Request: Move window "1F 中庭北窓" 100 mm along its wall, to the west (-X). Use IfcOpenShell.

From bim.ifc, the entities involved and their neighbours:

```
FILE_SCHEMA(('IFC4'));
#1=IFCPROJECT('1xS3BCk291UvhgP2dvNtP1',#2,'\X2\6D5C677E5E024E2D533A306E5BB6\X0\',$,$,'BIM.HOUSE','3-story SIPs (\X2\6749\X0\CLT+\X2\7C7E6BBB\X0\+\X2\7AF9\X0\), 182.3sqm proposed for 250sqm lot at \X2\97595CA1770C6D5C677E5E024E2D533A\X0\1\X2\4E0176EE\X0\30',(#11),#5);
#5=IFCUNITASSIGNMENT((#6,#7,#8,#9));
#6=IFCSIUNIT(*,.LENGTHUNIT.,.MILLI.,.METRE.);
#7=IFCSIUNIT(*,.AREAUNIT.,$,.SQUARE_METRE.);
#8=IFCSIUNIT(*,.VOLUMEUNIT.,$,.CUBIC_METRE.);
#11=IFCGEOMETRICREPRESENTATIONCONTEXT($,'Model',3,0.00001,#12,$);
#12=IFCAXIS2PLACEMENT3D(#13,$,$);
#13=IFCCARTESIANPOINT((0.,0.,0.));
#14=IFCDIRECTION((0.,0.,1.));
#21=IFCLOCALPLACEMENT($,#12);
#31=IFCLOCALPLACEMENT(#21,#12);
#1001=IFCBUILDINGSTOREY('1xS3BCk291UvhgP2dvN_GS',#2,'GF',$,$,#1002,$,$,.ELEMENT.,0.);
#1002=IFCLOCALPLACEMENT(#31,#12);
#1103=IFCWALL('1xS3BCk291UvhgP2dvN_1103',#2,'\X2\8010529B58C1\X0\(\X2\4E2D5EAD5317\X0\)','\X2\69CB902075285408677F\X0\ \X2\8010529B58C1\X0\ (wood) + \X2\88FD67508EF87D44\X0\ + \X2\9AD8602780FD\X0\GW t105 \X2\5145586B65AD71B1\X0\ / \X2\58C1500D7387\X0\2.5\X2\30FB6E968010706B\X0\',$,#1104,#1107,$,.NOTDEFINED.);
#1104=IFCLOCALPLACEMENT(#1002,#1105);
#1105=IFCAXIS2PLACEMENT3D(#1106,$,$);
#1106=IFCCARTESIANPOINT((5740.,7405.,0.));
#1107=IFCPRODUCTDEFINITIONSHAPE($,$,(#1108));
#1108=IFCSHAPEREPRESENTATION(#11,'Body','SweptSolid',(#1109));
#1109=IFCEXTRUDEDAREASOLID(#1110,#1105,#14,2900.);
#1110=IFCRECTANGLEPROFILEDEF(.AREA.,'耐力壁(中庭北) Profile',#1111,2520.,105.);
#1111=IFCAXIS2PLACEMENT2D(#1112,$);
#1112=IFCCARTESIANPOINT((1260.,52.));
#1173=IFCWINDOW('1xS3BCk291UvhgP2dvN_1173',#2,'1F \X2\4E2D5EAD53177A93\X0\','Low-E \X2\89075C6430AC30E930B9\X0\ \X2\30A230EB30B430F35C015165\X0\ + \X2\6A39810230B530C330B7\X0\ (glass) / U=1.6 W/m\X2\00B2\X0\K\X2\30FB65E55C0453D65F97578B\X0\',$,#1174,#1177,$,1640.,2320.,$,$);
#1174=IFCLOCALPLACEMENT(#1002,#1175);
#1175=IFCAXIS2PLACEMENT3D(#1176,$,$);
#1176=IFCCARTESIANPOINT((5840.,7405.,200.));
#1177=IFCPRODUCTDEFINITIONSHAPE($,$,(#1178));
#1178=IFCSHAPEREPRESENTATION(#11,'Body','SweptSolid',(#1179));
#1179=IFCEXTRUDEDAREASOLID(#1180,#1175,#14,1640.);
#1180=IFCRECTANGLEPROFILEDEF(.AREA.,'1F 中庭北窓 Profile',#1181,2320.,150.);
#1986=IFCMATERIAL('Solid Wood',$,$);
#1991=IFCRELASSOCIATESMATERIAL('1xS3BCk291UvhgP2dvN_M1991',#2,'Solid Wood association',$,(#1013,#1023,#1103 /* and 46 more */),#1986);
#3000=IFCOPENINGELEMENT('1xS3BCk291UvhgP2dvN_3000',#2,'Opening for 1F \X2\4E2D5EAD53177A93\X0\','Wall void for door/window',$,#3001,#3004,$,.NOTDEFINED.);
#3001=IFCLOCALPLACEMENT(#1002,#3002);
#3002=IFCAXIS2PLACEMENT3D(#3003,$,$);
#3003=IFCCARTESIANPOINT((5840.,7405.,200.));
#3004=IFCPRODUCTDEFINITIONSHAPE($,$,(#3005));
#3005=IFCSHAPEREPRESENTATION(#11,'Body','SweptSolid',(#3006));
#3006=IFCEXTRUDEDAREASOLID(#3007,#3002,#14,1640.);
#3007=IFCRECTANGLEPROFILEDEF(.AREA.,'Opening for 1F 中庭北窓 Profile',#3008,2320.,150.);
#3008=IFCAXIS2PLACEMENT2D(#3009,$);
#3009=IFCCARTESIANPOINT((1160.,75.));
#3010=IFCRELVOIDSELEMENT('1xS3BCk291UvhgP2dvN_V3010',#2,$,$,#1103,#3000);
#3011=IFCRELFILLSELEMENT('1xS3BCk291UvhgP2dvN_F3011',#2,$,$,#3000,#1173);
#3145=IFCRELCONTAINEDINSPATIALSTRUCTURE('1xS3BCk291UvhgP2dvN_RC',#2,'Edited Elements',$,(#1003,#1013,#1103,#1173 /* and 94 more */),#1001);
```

```python
import ifcopenshell
import ifcopenshell.api.geometry
import ifcopenshell.util.placement

model = ifcopenshell.open("bim.ifc")

window = model.by_id(1173)
opening = window.FillsVoids[0].RelatingOpeningElement
wall = opening.VoidsElements[0].RelatingBuildingElement

wall_matrix = ifcopenshell.util.placement.get_local_placement(wall.ObjectPlacement)
shift = wall_matrix[:3, 0] * -100.0
before = ifcopenshell.util.placement.get_local_placement(window.ObjectPlacement)[:3, 3].copy()

# The window is not placed relative to its opening, so move both.
for product in (opening, window):
    matrix = ifcopenshell.util.placement.get_local_placement(product.ObjectPlacement)
    matrix[:3, 3] += shift
    ifcopenshell.api.geometry.edit_object_placement(model, product=product, matrix=matrix, is_si=False)

after = ifcopenshell.util.placement.get_local_placement(window.ObjectPlacement)[:3, 3]
print("window moved by", (after - before).round(3) + 0.0)

model.write("bim_rev.ifc")
```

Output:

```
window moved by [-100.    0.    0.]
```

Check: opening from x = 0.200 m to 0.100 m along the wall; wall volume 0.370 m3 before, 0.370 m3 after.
